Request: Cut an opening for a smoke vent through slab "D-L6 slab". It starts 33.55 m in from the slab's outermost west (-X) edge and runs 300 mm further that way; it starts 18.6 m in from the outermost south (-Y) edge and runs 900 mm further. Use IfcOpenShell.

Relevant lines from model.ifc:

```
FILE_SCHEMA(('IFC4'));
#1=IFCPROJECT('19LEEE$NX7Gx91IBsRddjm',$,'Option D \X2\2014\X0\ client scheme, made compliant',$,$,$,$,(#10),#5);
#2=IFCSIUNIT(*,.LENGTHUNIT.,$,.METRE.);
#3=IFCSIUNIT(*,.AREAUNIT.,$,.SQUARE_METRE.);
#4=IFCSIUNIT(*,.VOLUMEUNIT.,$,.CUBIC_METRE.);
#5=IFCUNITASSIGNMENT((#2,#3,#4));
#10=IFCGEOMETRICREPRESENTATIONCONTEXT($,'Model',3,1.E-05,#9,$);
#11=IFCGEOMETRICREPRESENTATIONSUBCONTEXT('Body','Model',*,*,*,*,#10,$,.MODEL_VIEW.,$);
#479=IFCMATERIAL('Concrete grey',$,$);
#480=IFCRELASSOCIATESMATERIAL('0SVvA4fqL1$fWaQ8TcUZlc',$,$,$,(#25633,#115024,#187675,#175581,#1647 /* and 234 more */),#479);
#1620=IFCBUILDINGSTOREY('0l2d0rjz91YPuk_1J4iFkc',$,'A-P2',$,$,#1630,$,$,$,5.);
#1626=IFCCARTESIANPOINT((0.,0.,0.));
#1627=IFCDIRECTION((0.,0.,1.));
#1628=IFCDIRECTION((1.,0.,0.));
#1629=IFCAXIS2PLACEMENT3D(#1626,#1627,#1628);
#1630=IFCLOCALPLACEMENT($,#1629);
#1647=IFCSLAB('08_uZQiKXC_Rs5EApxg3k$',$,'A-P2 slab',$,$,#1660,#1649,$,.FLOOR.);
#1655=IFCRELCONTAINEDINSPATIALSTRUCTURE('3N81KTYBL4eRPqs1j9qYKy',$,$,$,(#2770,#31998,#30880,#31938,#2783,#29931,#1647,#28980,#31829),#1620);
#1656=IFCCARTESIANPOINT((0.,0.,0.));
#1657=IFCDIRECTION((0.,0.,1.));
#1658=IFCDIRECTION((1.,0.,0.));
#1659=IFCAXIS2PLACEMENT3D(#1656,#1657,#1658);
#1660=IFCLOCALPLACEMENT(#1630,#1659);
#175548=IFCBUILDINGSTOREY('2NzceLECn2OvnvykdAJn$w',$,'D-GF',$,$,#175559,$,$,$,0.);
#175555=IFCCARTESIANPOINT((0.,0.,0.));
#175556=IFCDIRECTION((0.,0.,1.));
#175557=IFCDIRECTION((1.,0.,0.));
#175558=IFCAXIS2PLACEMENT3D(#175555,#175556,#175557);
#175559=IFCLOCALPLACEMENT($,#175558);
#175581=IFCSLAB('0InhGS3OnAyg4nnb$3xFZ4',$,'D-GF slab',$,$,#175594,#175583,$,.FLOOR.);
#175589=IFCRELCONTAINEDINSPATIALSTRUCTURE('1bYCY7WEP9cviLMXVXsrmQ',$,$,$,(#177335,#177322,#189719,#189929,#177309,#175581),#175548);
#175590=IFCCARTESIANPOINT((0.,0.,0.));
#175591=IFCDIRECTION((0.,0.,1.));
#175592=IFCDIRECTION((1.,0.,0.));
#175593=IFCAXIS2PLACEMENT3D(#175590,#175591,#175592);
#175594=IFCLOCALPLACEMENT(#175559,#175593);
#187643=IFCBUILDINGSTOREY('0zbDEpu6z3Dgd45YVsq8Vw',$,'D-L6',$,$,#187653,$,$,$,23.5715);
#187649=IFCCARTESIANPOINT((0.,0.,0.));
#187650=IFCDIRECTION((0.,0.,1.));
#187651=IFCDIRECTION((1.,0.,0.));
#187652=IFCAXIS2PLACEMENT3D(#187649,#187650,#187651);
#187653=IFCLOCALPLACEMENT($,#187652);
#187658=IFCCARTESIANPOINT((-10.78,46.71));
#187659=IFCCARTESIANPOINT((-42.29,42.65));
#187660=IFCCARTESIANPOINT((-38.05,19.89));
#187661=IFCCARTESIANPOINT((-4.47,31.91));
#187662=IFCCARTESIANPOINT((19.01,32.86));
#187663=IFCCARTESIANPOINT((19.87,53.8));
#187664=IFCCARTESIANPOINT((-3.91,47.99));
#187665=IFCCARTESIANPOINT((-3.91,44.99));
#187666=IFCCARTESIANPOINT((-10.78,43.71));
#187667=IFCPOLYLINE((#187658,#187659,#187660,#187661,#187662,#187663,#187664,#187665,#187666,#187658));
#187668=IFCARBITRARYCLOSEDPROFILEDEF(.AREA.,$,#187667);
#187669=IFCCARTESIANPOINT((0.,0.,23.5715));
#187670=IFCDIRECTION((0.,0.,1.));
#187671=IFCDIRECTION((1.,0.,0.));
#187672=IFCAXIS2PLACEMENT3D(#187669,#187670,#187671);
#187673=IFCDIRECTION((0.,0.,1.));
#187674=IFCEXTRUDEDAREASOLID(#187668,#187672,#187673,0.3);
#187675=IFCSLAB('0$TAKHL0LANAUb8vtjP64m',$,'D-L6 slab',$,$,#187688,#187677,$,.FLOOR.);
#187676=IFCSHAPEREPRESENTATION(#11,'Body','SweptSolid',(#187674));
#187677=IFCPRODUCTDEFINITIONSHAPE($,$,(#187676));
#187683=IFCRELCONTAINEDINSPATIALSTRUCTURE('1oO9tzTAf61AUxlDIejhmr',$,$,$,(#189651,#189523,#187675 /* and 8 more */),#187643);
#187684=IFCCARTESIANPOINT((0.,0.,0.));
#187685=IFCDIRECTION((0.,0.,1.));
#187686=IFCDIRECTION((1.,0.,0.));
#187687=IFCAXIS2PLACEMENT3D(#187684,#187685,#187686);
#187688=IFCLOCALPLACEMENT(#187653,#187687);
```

```python
import numpy as np
import ifcopenshell
import ifcopenshell.api.feature
import ifcopenshell.api.geometry
import ifcopenshell.api.root
import ifcopenshell.geom
import ifcopenshell.util.placement
import ifcopenshell.util.representation
import ifcopenshell.util.shape
import ifcopenshell.util.unit

model = ifcopenshell.open("model.ifc")
unit_scale = ifcopenshell.util.unit.calculate_unit_scale(model)
settings = ifcopenshell.geom.settings()


def volume(element):
    """Net volume in cubic metres, openings subtracted."""
    shape = ifcopenshell.geom.create_shape(settings, element)
    return ifcopenshell.util.shape.get_volume(shape.geometry)


slab = model.by_guid("0$TAKHL0LANAUb8vtjP64m")
before = volume(slab)

# Extent in the slab's own axes, in metres. The edges named are its -X and -Y sides.
slab_shape = ifcopenshell.geom.create_shape(settings, slab)
vertices = ifcopenshell.util.shape.get_vertices(slab_shape.geometry)
x_min, y_min, bottom = vertices.min(axis=0)
top = vertices[:, 2].max()

opening = ifcopenshell.api.root.create_entity(model, ifc_class="IfcOpeningElement", name="Smoke vent opening", predefined_type="OPENING")
context = ifcopenshell.util.representation.get_context(model, "Model", "Body", "MODEL_VIEW")
width, depth = 0.3, 0.9
outline = [(0.0, 0.0), (width, 0.0), (width, depth), (0.0, depth), (0.0, 0.0)]
# Overshoot both faces by 50 mm so the cut is clean.
shape = ifcopenshell.api.geometry.add_slab_representation(
    model, context=context, depth=top - bottom + 0.1, polyline=outline
)
ifcopenshell.api.geometry.assign_representation(model, product=opening, representation=shape)

matrix = ifcopenshell.util.placement.get_local_placement(slab.ObjectPlacement)
matrix[:, 3] = matrix @ np.append(np.array([x_min + 33.55, y_min + 18.6, bottom - 0.05]) / unit_scale, 1.0)
ifcopenshell.api.geometry.edit_object_placement(model, product=opening, matrix=matrix, is_si=False)
ifcopenshell.api.feature.add_feature(model, feature=opening, element=slab)

after = volume(slab)

print(f"slab volume {before:.3f} -> {after:.3f} m3")

model.write("model-out.ifc")
```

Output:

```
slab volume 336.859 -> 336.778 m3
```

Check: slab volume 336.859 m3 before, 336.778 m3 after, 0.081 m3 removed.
